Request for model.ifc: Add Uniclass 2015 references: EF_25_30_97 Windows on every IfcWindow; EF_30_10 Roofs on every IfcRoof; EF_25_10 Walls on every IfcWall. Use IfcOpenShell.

First a look at what the model holds.

```python
import ifcopenshell

model = ifcopenshell.open("model.ifc")
print(model.schema)
print("classifications:", [c.Name for c in model.by_type("IfcClassification")])
for ifc_class in ("IfcDoor", "IfcRoof", "IfcStair", "IfcWall", "IfcWindow"):
    print(ifc_class, len(model.by_type(ifc_class)))
```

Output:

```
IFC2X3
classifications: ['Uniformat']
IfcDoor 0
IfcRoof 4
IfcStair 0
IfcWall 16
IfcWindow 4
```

```python
import ifcopenshell
import ifcopenshell.api.classification

model = ifcopenshell.open("model.ifc")

# IFC2X3 requires Source and Edition and has no link from the project to the system.
system = model.create_entity("IfcClassification", Source="NBS", Edition="2015", Name="Uniclass 2015")

codes = {
    "IfcWindow": ("EF_25_30_97", "Windows"),
    "IfcRoof": ("EF_30_10", "Roofs"),
    "IfcWall": ("EF_25_10", "Walls"),
}
for ifc_class, (code, name) in codes.items():
    products = model.by_type(ifc_class)
    ifcopenshell.api.classification.add_reference(
        model, products=products, classification=system, identification=code, name=name
    )
    print(code, len(products))

model.write("model_rev.ifc")
```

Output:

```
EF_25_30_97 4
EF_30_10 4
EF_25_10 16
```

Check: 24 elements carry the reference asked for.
